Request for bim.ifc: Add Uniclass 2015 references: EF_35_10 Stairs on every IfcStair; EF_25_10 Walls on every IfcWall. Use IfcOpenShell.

First a look at what the model holds.

```python
import ifcopenshell

model = ifcopenshell.open("bim.ifc")
print(model.schema)
print("classifications:", [c.Name for c in model.by_type("IfcClassification")])
for ifc_class in ("IfcDoor", "IfcRoof", "IfcStair", "IfcWall", "IfcWindow"):
    print(ifc_class, len(model.by_type(ifc_class)))
```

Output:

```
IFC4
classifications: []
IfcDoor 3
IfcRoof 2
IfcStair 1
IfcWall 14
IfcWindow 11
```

```python
import ifcopenshell
import ifcopenshell.api.classification

model = ifcopenshell.open("bim.ifc")

system = ifcopenshell.api.classification.add_classification(model, classification="Uniclass 2015")

codes = {
    "IfcStair": ("EF_35_10", "Stairs"),
    "IfcWall": ("EF_25_10", "Walls"),
}
for ifc_class, (code, name) in codes.items():
    products = model.by_type(ifc_class)
    ifcopenshell.api.classification.add_reference(
        model, products=products, classification=system, identification=code, name=name
    )
    print(code, len(products))

model.write("bim_updated.ifc")
```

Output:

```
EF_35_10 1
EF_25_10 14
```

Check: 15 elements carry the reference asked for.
